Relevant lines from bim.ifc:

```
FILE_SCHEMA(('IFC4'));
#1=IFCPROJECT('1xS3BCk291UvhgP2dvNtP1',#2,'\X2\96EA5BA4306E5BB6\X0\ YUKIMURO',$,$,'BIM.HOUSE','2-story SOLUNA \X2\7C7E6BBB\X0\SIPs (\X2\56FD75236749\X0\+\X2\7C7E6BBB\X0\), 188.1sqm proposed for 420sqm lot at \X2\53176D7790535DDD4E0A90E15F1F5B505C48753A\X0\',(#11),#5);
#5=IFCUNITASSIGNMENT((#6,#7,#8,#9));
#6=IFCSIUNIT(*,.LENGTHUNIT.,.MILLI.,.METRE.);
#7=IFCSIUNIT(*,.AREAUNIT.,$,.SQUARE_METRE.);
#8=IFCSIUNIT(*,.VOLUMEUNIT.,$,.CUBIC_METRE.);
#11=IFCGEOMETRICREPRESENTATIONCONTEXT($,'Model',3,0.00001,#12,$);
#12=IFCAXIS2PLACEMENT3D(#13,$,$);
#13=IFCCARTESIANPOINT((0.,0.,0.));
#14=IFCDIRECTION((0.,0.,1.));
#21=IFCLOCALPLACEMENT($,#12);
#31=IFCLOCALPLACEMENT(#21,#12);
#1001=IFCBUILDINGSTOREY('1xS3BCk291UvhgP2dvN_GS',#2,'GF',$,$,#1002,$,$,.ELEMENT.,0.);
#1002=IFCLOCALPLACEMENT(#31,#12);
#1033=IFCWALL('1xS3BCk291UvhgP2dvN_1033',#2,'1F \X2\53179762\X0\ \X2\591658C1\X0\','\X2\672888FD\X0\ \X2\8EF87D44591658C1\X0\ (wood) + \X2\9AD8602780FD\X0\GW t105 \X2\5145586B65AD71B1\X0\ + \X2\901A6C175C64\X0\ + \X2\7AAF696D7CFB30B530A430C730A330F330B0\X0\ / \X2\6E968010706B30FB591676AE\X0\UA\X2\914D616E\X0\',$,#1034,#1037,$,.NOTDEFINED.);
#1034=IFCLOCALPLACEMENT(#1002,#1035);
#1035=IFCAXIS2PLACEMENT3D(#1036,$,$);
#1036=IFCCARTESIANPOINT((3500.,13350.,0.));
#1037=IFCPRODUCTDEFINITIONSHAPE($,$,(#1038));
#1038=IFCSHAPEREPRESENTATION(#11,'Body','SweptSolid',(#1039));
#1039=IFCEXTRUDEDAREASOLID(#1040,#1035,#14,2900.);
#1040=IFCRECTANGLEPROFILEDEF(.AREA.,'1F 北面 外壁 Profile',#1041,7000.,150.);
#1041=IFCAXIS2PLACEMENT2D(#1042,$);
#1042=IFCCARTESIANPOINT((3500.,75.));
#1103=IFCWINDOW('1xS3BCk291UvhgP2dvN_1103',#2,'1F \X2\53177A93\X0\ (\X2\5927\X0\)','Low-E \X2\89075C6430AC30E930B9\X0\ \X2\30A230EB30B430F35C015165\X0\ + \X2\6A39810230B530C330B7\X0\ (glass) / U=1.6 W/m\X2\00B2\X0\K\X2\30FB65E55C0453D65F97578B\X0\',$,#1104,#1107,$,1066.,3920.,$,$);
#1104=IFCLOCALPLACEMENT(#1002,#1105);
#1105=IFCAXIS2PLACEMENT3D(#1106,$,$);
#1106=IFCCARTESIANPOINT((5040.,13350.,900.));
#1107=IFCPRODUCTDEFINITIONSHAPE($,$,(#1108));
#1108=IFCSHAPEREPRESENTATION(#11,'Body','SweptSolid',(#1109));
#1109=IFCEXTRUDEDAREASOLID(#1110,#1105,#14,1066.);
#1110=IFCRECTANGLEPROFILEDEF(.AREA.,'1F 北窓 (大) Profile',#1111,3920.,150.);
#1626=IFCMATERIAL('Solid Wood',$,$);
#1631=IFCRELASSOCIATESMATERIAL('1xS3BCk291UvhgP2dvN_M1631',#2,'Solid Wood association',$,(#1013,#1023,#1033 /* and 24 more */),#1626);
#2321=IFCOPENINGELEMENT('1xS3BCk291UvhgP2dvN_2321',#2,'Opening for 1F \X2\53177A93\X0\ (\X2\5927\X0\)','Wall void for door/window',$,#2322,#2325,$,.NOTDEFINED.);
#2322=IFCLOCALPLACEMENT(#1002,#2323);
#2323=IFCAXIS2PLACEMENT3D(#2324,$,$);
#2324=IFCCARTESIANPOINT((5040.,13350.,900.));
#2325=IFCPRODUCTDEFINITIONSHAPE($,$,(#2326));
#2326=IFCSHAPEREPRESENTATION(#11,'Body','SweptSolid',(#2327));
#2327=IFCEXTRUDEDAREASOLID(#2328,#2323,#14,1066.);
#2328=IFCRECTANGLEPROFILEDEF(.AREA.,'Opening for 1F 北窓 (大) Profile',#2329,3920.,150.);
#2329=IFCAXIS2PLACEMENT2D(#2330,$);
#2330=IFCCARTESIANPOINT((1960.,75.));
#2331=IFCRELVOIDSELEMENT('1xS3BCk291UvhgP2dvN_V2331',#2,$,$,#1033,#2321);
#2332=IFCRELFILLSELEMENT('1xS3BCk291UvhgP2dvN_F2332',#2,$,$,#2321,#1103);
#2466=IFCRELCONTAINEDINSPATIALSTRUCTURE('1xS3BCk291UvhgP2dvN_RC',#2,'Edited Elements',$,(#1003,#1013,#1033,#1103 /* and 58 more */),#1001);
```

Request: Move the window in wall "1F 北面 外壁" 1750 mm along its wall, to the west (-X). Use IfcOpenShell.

```python
import ifcopenshell
import ifcopenshell.api.geometry
import ifcopenshell.util.placement

model = ifcopenshell.open("bim.ifc")

window = model.by_guid("1xS3BCk291UvhgP2dvN_1103")
opening = window.FillsVoids[0].RelatingOpeningElement
wall = opening.VoidsElements[0].RelatingBuildingElement

wall_matrix = ifcopenshell.util.placement.get_local_placement(wall.ObjectPlacement)
shift = wall_matrix[:3, 0] * -1750.0
before = ifcopenshell.util.placement.get_local_placement(window.ObjectPlacement)[:3, 3].copy()

# The window is not placed relative to its opening, so move both.
for product in (opening, window):
    matrix = ifcopenshell.util.placement.get_local_placement(product.ObjectPlacement)
    matrix[:3, 3] += shift
    ifcopenshell.api.geometry.edit_object_placement(model, product=product, matrix=matrix, is_si=False)

after = ifcopenshell.util.placement.get_local_placement(window.ObjectPlacement)[:3, 3]
print("window moved by", (after - before).round(3) + 0.0)

model.write("bim_edited.ifc")
```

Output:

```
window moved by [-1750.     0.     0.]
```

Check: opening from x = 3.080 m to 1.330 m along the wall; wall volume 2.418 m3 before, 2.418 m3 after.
